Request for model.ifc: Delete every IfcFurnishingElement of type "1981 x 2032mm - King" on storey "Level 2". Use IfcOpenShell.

First a look at what the model holds.

```python
import ifcopenshell
import ifcopenshell.util.element

model = ifcopenshell.open("model.ifc")
print(model.schema)
storey = next(s for s in model.by_type("IfcBuildingStorey") if s.Name == "Level 2")
furniture = [e for e in ifcopenshell.util.element.get_decomposition(storey) if e.is_a("IfcFurnishingElement")]
seen = {}
for e in furniture:
    element_type = ifcopenshell.util.element.get_type(e)
    name = element_type.Name if element_type not in (None, e) else None
    seen[name] = seen.get(name, 0) + 1
for name, count in sorted(seen.items(), key=str):
    print(count, "x", name)
```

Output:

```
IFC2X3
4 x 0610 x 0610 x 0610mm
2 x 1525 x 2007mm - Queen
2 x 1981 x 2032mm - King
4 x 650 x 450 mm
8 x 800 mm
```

```python
import ifcopenshell
import ifcopenshell.api.root
import ifcopenshell.util.element

model = ifcopenshell.open("model.ifc")

storey = next(s for s in model.by_type("IfcBuildingStorey") if s.Name == "Level 2")
furniture = [e for e in ifcopenshell.util.element.get_decomposition(storey) if e.is_a("IfcFurnishingElement")]
targets = [e for e in furniture if (t := ifcopenshell.util.element.get_type(e)) not in (None, e) and t.Name == "1981 x 2032mm - King"]

for e in targets:
    ifcopenshell.api.root.remove_product(model, product=e)
print(len(targets), "removed")

model.write("model-out.ifc")
```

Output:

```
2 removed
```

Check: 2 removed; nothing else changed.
